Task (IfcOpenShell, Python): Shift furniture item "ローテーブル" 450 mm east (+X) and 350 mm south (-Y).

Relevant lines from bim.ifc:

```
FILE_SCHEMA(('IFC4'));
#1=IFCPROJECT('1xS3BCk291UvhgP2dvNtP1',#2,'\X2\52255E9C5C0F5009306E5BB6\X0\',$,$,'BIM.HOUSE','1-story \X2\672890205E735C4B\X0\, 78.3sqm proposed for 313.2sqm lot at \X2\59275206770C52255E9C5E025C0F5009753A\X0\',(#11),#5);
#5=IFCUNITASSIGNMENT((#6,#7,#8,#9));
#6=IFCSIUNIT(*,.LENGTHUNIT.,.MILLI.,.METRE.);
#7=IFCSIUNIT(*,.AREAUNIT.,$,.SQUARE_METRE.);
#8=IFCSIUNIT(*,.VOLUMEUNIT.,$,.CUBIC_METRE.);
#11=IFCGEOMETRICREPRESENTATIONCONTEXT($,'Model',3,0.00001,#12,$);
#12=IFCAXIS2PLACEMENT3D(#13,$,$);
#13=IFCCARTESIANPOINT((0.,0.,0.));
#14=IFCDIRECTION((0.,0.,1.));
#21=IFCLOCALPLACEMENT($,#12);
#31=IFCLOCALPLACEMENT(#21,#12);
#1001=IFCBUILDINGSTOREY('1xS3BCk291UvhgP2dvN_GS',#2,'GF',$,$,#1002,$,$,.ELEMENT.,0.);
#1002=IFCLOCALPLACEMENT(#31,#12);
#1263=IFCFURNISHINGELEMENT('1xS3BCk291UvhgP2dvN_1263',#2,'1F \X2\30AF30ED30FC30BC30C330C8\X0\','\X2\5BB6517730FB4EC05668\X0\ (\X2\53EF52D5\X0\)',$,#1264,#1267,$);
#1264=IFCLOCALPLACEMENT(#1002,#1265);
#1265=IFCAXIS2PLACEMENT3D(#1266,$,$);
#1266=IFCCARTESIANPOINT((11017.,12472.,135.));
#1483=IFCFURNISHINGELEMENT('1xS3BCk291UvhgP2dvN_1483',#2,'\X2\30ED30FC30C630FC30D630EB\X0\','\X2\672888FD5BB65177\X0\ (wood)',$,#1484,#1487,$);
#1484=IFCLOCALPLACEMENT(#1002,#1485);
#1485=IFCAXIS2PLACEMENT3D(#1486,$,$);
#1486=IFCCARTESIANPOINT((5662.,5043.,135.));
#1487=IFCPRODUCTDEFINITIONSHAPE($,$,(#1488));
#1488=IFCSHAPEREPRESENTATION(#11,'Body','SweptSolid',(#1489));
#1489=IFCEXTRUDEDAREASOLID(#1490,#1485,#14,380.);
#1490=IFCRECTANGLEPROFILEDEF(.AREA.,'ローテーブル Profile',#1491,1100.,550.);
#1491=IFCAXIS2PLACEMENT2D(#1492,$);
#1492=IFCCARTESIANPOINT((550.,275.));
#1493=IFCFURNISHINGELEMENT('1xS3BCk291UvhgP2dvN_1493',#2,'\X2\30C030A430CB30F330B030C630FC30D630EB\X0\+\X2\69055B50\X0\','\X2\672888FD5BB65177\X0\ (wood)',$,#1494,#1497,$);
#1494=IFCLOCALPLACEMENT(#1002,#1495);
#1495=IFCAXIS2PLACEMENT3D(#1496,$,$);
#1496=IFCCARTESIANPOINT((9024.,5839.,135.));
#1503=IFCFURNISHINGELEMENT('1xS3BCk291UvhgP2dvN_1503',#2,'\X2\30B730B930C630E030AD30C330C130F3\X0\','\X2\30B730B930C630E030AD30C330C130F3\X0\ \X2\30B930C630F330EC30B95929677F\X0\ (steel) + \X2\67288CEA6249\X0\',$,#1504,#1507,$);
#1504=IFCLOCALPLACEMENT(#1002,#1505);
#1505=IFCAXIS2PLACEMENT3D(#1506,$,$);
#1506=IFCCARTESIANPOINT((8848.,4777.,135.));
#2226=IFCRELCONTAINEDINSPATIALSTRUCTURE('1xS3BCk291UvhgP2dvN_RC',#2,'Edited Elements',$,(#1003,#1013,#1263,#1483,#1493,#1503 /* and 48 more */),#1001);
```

```python
import ifcopenshell
import ifcopenshell.api.geometry
import ifcopenshell.util.placement
import ifcopenshell.util.unit

model = ifcopenshell.open("bim.ifc")
unit_scale = ifcopenshell.util.unit.calculate_unit_scale(model)

item = model.by_id(1483)
matrix = ifcopenshell.util.placement.get_local_placement(item.ObjectPlacement)
matrix[0, 3] += 0.45 / unit_scale
matrix[1, 3] -= 0.35 / unit_scale
ifcopenshell.api.geometry.edit_object_placement(model, product=item, matrix=matrix, is_si=False)

print(ifcopenshell.util.placement.get_local_placement(item.ObjectPlacement).round(3) + 0.0)

model.write("bim_updated.ifc")
```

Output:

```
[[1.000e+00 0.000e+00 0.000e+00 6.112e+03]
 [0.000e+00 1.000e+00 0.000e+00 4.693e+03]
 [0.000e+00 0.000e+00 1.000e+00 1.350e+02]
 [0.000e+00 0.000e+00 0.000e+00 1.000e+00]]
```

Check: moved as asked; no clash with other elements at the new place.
